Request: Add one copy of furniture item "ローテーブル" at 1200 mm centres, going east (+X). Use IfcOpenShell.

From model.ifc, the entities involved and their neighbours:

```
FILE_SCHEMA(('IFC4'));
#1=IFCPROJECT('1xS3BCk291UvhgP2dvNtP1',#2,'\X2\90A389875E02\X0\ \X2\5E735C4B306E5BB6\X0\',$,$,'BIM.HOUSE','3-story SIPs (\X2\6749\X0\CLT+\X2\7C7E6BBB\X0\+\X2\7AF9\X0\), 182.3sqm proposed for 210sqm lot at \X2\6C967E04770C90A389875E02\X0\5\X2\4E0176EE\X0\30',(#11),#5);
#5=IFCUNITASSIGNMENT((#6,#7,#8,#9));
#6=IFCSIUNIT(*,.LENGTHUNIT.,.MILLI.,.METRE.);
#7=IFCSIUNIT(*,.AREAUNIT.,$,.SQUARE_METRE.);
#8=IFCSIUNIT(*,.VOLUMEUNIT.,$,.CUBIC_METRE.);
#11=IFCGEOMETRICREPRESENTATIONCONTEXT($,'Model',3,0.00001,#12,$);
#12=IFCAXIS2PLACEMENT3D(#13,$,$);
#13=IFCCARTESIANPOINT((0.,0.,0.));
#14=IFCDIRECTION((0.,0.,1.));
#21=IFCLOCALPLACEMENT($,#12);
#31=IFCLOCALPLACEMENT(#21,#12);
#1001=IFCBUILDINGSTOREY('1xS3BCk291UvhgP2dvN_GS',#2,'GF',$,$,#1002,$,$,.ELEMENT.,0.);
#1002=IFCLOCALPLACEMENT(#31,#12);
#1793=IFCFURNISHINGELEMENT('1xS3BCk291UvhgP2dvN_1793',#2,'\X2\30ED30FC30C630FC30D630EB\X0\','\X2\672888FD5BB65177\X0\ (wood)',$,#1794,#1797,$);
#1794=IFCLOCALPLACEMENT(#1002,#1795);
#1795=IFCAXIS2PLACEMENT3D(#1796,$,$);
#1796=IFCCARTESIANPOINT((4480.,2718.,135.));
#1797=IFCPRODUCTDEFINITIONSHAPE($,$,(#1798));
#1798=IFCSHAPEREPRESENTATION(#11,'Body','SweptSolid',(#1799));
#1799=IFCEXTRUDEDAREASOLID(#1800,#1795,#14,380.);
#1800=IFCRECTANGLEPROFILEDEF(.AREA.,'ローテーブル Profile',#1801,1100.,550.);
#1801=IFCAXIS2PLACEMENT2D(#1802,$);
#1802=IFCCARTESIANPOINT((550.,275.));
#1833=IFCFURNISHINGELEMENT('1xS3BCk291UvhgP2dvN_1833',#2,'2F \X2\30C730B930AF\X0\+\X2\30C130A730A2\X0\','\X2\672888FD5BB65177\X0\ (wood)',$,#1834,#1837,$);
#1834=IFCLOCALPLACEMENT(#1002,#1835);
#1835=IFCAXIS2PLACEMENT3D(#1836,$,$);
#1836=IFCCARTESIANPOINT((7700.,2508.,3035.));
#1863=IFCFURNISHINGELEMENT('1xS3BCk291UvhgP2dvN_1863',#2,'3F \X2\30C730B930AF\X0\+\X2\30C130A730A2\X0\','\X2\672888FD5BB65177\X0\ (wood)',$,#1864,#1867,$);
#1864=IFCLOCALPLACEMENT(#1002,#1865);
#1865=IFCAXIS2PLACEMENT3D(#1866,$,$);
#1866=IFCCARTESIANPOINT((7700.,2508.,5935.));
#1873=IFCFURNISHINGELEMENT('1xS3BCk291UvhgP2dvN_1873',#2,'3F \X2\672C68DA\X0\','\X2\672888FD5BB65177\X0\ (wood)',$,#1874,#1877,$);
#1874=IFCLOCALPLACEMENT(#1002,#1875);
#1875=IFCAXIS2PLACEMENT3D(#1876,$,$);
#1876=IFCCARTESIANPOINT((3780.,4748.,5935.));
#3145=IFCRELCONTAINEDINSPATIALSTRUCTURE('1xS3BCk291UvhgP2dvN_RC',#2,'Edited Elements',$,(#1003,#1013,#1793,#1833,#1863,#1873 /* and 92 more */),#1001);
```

```python
import numpy as np
import ifcopenshell
import ifcopenshell.api.geometry
import ifcopenshell.api.root
import ifcopenshell.util.element
import ifcopenshell.util.placement

model = ifcopenshell.open("model.ifc")


def reuse_history(source, copy):
    """copy_class also copies each property set's owner history, people and application; keep the originals."""
    for rel in copy.IsDefinedBy:
        if rel.is_a("IfcRelDefinesByProperties") and (history := rel.RelatingPropertyDefinition.OwnerHistory):
            rel.RelatingPropertyDefinition.OwnerHistory = source.OwnerHistory
            ifcopenshell.util.element.remove_deep2(model, history)


source = model.by_guid("1xS3BCk291UvhgP2dvN_1793")
base = ifcopenshell.util.placement.get_local_placement(source.ObjectPlacement)
step = np.array([1.0, 0.0, 0.0]) * 1200.0

for i in range(1, 2):
    copy = ifcopenshell.api.root.copy_class(model, product=source)
    copy.Representation = ifcopenshell.util.element.copy_deep(
        model, source.Representation, exclude=["IfcGeometricRepresentationContext", "IfcRepresentationMap"]
    )
    reuse_history(source, copy)
    matrix = base.copy()
    matrix[:3, 3] += i * step
    print("added at", matrix[:3, 3].round(3) + 0.0)
    ifcopenshell.api.geometry.edit_object_placement(model, product=copy, matrix=matrix, is_si=False)

model.write("model_rev.ifc")
```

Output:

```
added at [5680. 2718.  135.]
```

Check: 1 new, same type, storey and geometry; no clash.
